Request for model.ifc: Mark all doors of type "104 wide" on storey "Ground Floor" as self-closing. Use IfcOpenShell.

First a look at what the model holds.

```python
import ifcopenshell
import ifcopenshell.util.element

model = ifcopenshell.open("model.ifc")
print(model.schema)
storey = next(s for s in model.by_type("IfcBuildingStorey") if s.Name == "Ground Floor")
doors = [e for e in ifcopenshell.util.element.get_decomposition(storey) if e.is_a("IfcDoor")]
seen = {}
for e in doors:
    element_type = ifcopenshell.util.element.get_type(e)
    key = (element_type.Name if element_type != e and element_type else None, ifcopenshell.util.element.get_pset(e, "Pset_DoorCommon", "SelfClosing"))
    seen[key] = seen.get(key, 0) + 1
for (name, value), count in sorted(seen.items(), key=str):
    print(count, "x", name, "|", value)
```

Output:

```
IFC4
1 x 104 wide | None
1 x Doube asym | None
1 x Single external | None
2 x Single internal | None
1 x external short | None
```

```python
import ifcopenshell
import ifcopenshell.api.pset
import ifcopenshell.util.element

model = ifcopenshell.open("model.ifc")

storey = next(s for s in model.by_type("IfcBuildingStorey") if s.Name == "Ground Floor")
doors = [e for e in ifcopenshell.util.element.get_decomposition(storey) if e.is_a("IfcDoor")]

count = 0
for e in doors:
    element_type = ifcopenshell.util.element.get_type(e)
    if element_type in (None, e) or element_type.Name != "104 wide":
        continue
    # add_pset returns the element's existing set when there is one.
    pset = ifcopenshell.api.pset.add_pset(model, product=e, name="Pset_DoorCommon")
    ifcopenshell.api.pset.edit_pset(model, pset=pset, properties={"SelfClosing": True})
    count += 1

print(count, "doors updated")

model.write("model_edited.ifc")
```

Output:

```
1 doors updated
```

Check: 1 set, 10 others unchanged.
